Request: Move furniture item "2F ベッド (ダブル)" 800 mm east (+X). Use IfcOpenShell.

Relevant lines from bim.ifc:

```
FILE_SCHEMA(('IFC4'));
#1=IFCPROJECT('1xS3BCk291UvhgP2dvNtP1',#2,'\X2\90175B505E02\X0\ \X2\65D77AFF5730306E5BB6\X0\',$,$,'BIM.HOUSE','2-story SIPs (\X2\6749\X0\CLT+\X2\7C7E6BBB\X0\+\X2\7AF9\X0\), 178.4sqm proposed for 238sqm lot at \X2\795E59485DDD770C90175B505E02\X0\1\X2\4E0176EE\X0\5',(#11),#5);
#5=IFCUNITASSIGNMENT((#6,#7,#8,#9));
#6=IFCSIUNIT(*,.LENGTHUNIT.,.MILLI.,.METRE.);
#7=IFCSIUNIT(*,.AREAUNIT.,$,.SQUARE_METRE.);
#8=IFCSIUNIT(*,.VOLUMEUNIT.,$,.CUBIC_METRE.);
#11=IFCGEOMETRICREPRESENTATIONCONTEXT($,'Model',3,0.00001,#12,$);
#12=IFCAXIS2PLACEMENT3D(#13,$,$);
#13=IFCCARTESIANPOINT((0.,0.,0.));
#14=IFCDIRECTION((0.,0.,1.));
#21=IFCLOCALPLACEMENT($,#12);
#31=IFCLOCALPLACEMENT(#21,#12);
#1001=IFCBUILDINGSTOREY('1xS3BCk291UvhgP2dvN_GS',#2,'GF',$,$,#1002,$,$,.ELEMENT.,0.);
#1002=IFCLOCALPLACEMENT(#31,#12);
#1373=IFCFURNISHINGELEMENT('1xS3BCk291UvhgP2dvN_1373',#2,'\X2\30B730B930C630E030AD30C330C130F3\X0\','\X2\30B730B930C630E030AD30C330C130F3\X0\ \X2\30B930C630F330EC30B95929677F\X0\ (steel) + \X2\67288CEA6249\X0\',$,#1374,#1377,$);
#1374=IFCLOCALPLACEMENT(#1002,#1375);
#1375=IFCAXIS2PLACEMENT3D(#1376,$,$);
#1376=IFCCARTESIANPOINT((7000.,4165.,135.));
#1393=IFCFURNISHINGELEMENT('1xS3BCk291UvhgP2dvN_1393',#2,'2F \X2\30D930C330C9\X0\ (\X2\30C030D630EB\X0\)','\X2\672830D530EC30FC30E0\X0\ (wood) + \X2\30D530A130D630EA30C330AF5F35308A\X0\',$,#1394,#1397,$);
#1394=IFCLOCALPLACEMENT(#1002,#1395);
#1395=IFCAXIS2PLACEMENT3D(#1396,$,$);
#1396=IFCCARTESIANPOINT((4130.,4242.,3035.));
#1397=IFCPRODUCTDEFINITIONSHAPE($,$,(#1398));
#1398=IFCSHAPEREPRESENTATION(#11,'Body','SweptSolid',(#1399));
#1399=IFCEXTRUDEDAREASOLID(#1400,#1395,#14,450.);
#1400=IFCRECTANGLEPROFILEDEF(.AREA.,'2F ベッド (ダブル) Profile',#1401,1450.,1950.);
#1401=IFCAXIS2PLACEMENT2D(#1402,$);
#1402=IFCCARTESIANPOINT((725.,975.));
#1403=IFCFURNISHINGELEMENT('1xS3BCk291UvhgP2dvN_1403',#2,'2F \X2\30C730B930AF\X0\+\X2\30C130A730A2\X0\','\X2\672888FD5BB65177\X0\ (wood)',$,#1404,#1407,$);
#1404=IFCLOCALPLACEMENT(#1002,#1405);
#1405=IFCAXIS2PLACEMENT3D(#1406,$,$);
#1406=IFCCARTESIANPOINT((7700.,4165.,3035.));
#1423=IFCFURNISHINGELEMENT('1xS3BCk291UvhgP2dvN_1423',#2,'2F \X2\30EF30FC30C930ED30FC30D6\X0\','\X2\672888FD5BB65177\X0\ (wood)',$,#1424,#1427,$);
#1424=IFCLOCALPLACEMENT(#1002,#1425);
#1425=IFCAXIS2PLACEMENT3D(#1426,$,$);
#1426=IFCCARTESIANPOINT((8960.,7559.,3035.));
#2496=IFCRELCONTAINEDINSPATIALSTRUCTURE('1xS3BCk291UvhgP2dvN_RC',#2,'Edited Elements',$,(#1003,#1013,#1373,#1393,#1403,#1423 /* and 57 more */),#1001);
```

```python
import ifcopenshell
import ifcopenshell.api.geometry
import ifcopenshell.util.placement
import ifcopenshell.util.unit

model = ifcopenshell.open("bim.ifc")
unit_scale = ifcopenshell.util.unit.calculate_unit_scale(model)

item = model.by_guid("1xS3BCk291UvhgP2dvN_1393")
matrix = ifcopenshell.util.placement.get_local_placement(item.ObjectPlacement)
matrix[0, 3] += 0.8 / unit_scale
ifcopenshell.api.geometry.edit_object_placement(model, product=item, matrix=matrix, is_si=False)

print(ifcopenshell.util.placement.get_local_placement(item.ObjectPlacement).round(3) + 0.0)

model.write("bim_v2.ifc")
```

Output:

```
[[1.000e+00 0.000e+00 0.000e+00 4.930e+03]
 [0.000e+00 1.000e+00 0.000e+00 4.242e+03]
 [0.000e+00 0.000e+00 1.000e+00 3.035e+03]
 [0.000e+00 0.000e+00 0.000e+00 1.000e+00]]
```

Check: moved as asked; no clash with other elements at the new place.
